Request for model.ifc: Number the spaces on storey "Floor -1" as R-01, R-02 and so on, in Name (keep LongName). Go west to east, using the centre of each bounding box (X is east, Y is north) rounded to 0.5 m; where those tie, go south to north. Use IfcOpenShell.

First a look at what the model holds.

```python
import ifcopenshell
import ifcopenshell.util.element
import ifcopenshell.util.placement

model = ifcopenshell.open("model.ifc")
print(model.schema)
storey = next(s for s in model.by_type("IfcBuildingStorey") if s.Name == "Floor -1")
spaces = [e for e in ifcopenshell.util.element.get_decomposition(storey) if e.is_a("IfcSpace")]
for e in sorted(spaces, key=lambda e: e.id()):
    origin = ifcopenshell.util.placement.get_local_placement(e.ObjectPlacement)[:3, 3]
    print(e.id(), e.Name, e.LongName, origin.round(2) + 0.0, sep=" | ")
```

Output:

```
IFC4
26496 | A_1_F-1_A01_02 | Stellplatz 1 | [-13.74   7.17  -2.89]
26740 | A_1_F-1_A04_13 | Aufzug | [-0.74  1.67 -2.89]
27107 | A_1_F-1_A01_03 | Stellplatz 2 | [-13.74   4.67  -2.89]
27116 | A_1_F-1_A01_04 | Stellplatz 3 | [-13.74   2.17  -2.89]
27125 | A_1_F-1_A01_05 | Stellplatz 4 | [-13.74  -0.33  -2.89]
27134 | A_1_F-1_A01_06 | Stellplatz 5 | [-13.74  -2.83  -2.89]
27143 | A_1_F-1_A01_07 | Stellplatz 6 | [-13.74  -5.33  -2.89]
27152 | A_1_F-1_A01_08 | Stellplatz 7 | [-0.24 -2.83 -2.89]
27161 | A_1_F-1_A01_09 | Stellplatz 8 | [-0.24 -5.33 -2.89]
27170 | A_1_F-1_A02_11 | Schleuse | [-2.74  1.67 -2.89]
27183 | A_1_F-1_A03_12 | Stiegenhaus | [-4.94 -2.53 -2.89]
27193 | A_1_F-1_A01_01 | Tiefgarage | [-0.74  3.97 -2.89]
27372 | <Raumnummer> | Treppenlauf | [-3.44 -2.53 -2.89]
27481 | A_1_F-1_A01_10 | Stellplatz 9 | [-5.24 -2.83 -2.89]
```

```python
import ifcopenshell
import ifcopenshell.geom
import ifcopenshell.util.element
import ifcopenshell.util.shape

model = ifcopenshell.open("model.ifc")
settings = ifcopenshell.geom.settings()
settings.set("use-world-coords", True)


def centre(element):
    shape = ifcopenshell.geom.create_shape(settings, element)
    return ifcopenshell.util.shape.get_bbox_centroid(shape.geometry)


storey = next(s for s in model.by_type("IfcBuildingStorey") if s.Name == "Floor -1")
spaces = [e for e in ifcopenshell.util.element.get_decomposition(storey) if e.is_a("IfcSpace")]

# Insertion points can sit at a corner or the storey origin, so sort by the geometry (in metres).
centres = {e: centre(e) for e in spaces}
spaces.sort(key=lambda e: (round(centres[e][0] / 0.5), centres[e][1]))

for i, e in enumerate(spaces, start=1):
    number = f"R-{i:02d}"
    e.Name = number
    print(e.id(), number)

model.write("model_updated.ifc")
```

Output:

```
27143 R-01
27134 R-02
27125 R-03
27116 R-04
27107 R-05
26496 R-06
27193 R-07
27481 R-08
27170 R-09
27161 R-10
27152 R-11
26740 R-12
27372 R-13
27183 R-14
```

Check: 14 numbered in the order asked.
